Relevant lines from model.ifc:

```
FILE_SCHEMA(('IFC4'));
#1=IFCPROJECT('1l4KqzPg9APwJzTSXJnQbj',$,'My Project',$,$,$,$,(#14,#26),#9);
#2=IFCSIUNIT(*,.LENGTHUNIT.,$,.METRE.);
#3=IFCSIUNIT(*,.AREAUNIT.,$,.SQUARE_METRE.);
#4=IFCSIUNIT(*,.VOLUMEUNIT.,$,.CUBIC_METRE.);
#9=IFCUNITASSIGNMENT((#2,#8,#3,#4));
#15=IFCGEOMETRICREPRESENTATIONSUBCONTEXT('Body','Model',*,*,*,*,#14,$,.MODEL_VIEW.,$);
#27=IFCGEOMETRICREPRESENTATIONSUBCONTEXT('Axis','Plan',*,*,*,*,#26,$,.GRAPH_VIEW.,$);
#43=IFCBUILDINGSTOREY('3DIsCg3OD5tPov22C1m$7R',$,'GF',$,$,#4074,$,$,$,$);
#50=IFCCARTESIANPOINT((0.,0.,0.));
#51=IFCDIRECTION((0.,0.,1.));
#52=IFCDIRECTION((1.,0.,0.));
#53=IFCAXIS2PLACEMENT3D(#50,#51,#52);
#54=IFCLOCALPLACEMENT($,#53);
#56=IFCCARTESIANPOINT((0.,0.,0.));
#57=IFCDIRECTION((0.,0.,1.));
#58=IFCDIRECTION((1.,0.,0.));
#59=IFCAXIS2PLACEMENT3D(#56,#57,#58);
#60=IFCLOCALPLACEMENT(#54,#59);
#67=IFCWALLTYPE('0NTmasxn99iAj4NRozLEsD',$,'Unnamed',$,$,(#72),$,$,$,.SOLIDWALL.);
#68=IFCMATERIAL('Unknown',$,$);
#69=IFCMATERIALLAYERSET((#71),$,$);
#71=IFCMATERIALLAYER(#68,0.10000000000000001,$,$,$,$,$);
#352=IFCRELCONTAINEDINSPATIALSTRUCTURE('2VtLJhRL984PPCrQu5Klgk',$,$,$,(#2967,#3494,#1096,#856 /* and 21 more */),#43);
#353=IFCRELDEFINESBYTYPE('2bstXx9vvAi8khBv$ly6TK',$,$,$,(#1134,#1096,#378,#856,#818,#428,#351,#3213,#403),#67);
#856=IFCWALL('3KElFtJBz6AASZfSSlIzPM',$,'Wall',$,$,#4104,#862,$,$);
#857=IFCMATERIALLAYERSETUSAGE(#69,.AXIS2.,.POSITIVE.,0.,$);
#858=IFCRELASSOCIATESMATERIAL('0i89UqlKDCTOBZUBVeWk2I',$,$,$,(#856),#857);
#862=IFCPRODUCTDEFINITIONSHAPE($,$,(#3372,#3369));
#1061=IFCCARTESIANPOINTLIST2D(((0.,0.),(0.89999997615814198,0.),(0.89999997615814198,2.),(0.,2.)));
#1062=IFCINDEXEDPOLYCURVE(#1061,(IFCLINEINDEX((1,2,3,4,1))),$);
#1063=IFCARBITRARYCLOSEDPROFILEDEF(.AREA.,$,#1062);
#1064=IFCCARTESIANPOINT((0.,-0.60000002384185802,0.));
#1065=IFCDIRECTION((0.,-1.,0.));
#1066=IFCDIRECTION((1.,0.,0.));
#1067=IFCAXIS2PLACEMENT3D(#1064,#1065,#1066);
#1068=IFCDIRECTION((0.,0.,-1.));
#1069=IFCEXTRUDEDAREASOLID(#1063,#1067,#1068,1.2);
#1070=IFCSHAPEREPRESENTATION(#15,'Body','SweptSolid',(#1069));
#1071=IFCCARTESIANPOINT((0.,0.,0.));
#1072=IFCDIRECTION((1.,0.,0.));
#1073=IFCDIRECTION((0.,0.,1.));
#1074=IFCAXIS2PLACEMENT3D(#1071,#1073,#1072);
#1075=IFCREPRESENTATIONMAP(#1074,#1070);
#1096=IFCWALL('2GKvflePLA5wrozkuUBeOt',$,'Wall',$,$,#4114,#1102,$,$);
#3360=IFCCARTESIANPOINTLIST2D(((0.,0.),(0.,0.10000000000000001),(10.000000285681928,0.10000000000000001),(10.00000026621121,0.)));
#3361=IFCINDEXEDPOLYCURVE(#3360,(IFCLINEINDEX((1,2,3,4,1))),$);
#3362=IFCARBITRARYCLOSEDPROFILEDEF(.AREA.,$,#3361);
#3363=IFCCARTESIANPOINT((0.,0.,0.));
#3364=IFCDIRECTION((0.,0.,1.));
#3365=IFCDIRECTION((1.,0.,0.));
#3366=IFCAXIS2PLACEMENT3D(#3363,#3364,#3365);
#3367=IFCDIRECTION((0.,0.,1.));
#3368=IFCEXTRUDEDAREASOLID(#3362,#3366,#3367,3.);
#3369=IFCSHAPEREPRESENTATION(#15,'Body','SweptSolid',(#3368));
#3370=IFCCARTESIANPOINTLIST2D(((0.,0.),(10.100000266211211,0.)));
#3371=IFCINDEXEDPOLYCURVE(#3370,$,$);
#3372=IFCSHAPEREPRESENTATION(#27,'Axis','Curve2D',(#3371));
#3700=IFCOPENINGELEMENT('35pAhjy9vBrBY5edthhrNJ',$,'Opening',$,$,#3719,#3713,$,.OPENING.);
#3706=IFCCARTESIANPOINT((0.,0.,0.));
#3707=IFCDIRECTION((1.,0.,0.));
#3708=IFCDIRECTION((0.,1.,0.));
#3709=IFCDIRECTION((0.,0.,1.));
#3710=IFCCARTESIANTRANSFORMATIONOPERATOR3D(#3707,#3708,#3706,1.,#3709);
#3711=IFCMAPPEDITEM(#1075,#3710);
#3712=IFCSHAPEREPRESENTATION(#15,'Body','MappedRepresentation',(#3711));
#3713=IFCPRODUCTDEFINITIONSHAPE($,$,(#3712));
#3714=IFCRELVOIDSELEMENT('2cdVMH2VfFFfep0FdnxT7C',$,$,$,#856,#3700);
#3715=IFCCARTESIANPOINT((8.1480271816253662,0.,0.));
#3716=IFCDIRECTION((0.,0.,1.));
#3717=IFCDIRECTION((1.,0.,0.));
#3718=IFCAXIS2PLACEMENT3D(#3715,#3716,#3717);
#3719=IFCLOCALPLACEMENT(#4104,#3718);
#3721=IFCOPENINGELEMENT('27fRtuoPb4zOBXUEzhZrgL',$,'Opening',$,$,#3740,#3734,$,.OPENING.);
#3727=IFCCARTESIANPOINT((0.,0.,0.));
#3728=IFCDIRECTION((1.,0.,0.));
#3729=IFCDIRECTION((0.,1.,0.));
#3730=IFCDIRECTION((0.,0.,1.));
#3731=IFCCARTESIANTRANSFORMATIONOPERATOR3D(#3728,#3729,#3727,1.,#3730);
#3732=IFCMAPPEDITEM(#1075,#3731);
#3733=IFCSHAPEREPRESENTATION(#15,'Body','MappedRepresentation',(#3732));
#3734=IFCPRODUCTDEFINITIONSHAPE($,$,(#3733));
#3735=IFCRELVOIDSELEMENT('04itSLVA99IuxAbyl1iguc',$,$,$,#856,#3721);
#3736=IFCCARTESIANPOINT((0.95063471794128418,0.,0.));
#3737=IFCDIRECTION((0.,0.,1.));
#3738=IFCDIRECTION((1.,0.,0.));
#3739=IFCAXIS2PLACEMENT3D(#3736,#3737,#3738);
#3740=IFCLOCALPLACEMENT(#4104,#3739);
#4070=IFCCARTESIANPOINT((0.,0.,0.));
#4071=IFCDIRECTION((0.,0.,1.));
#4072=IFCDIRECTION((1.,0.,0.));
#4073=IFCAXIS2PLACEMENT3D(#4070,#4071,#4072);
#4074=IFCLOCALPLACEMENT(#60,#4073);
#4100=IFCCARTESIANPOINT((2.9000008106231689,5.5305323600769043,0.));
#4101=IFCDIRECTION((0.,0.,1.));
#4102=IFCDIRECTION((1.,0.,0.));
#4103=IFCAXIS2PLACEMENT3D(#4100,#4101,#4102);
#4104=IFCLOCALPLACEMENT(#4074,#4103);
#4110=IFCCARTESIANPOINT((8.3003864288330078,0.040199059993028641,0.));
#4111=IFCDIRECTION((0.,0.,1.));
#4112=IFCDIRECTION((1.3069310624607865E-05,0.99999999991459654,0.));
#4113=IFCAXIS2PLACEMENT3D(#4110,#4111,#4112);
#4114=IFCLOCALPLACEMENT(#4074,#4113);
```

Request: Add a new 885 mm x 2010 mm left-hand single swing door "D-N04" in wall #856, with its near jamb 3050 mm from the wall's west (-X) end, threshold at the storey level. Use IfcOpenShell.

```python
import numpy as np
import ifcopenshell
import ifcopenshell.api.feature
import ifcopenshell.api.geometry
import ifcopenshell.api.root
import ifcopenshell.api.spatial
import ifcopenshell.geom
import ifcopenshell.util.element
import ifcopenshell.util.placement
import ifcopenshell.util.representation
import ifcopenshell.util.shape
import ifcopenshell.util.unit

model = ifcopenshell.open("model.ifc")
unit_scale = ifcopenshell.util.unit.calculate_unit_scale(model)
settings = ifcopenshell.geom.settings()


def volume(element):
    """Net volume in cubic metres, openings subtracted."""
    shape = ifcopenshell.geom.create_shape(settings, element)
    return ifcopenshell.util.shape.get_volume(shape.geometry)


wall = model.by_guid("3KElFtJBz6AASZfSSlIzPM")
storey = ifcopenshell.util.element.get_container(wall, ifc_class="IfcBuildingStorey")
context = ifcopenshell.util.representation.get_context(model, "Model", "Body", "MODEL_VIEW")
before = volume(wall)

width, height, from_end, sill = 0.885, 2.01, 3.05, 0.0  # metres

# The wall runs along its own X axis, and the end named is its -X end.
wall_shape = ifcopenshell.geom.create_shape(settings, wall)
x, y, z = ifcopenshell.util.shape.get_vertices(wall_shape.geometry).T
start = x.min() + from_end
face, thickness = float(y.min()), float(y.max() - y.min())
wall_matrix = ifcopenshell.util.placement.get_local_placement(wall.ObjectPlacement)
level = ifcopenshell.util.placement.get_local_placement(storey.ObjectPlacement)[2, 3]


def in_wall(x, y):
    """Placement at x, y metres in the wall's axes, at sill height."""
    matrix = wall_matrix.copy()
    matrix[:, 3] = wall_matrix @ np.array([x / unit_scale, y / unit_scale, 0.0, 1.0])
    matrix[2, 3] = level + sill / unit_scale
    return matrix


# Opening: a box that overshoots both wall faces by 50 mm.
opening = ifcopenshell.api.root.create_entity(model, ifc_class="IfcOpeningElement", predefined_type="OPENING")
box = ifcopenshell.api.geometry.add_wall_representation(
    model, context=context, length=width, height=height, thickness=thickness + 0.1
)
ifcopenshell.api.geometry.assign_representation(model, product=opening, representation=box)
ifcopenshell.api.geometry.edit_object_placement(model, product=opening, matrix=in_wall(start, face - 0.05), is_si=False)
ifcopenshell.api.feature.add_feature(model, feature=opening, element=wall)

door = ifcopenshell.api.root.create_entity(model, ifc_class="IfcDoor", name="D-N04", predefined_type="DOOR")
door.OverallWidth, door.OverallHeight = width / unit_scale, height / unit_scale
door.OperationType = "SINGLE_SWING_LEFT"
body = ifcopenshell.api.geometry.add_door_representation(
    model,
    context=context,
    overall_width=door.OverallWidth,
    overall_height=door.OverallHeight,
    operation_type="SINGLE_SWING_LEFT",
    lining_properties={"LiningDepth": thickness / unit_scale, "ThresholdDepth": thickness / unit_scale},
)
ifcopenshell.api.geometry.assign_representation(model, product=door, representation=body)
ifcopenshell.api.spatial.assign_container(model, products=[door], relating_structure=storey)
ifcopenshell.api.feature.add_filling(model, opening=opening, element=door)

# The lining spans the wall, so the door starts at the wall face.
ifcopenshell.api.geometry.edit_object_placement(model, product=door, matrix=in_wall(start, face), is_si=False)

after = volume(wall)

print(f"wall volume {before:.3f} -> {after:.3f} m3")

model.write("model_rev.ifc")
```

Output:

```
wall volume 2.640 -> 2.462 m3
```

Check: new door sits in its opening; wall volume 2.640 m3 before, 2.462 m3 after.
